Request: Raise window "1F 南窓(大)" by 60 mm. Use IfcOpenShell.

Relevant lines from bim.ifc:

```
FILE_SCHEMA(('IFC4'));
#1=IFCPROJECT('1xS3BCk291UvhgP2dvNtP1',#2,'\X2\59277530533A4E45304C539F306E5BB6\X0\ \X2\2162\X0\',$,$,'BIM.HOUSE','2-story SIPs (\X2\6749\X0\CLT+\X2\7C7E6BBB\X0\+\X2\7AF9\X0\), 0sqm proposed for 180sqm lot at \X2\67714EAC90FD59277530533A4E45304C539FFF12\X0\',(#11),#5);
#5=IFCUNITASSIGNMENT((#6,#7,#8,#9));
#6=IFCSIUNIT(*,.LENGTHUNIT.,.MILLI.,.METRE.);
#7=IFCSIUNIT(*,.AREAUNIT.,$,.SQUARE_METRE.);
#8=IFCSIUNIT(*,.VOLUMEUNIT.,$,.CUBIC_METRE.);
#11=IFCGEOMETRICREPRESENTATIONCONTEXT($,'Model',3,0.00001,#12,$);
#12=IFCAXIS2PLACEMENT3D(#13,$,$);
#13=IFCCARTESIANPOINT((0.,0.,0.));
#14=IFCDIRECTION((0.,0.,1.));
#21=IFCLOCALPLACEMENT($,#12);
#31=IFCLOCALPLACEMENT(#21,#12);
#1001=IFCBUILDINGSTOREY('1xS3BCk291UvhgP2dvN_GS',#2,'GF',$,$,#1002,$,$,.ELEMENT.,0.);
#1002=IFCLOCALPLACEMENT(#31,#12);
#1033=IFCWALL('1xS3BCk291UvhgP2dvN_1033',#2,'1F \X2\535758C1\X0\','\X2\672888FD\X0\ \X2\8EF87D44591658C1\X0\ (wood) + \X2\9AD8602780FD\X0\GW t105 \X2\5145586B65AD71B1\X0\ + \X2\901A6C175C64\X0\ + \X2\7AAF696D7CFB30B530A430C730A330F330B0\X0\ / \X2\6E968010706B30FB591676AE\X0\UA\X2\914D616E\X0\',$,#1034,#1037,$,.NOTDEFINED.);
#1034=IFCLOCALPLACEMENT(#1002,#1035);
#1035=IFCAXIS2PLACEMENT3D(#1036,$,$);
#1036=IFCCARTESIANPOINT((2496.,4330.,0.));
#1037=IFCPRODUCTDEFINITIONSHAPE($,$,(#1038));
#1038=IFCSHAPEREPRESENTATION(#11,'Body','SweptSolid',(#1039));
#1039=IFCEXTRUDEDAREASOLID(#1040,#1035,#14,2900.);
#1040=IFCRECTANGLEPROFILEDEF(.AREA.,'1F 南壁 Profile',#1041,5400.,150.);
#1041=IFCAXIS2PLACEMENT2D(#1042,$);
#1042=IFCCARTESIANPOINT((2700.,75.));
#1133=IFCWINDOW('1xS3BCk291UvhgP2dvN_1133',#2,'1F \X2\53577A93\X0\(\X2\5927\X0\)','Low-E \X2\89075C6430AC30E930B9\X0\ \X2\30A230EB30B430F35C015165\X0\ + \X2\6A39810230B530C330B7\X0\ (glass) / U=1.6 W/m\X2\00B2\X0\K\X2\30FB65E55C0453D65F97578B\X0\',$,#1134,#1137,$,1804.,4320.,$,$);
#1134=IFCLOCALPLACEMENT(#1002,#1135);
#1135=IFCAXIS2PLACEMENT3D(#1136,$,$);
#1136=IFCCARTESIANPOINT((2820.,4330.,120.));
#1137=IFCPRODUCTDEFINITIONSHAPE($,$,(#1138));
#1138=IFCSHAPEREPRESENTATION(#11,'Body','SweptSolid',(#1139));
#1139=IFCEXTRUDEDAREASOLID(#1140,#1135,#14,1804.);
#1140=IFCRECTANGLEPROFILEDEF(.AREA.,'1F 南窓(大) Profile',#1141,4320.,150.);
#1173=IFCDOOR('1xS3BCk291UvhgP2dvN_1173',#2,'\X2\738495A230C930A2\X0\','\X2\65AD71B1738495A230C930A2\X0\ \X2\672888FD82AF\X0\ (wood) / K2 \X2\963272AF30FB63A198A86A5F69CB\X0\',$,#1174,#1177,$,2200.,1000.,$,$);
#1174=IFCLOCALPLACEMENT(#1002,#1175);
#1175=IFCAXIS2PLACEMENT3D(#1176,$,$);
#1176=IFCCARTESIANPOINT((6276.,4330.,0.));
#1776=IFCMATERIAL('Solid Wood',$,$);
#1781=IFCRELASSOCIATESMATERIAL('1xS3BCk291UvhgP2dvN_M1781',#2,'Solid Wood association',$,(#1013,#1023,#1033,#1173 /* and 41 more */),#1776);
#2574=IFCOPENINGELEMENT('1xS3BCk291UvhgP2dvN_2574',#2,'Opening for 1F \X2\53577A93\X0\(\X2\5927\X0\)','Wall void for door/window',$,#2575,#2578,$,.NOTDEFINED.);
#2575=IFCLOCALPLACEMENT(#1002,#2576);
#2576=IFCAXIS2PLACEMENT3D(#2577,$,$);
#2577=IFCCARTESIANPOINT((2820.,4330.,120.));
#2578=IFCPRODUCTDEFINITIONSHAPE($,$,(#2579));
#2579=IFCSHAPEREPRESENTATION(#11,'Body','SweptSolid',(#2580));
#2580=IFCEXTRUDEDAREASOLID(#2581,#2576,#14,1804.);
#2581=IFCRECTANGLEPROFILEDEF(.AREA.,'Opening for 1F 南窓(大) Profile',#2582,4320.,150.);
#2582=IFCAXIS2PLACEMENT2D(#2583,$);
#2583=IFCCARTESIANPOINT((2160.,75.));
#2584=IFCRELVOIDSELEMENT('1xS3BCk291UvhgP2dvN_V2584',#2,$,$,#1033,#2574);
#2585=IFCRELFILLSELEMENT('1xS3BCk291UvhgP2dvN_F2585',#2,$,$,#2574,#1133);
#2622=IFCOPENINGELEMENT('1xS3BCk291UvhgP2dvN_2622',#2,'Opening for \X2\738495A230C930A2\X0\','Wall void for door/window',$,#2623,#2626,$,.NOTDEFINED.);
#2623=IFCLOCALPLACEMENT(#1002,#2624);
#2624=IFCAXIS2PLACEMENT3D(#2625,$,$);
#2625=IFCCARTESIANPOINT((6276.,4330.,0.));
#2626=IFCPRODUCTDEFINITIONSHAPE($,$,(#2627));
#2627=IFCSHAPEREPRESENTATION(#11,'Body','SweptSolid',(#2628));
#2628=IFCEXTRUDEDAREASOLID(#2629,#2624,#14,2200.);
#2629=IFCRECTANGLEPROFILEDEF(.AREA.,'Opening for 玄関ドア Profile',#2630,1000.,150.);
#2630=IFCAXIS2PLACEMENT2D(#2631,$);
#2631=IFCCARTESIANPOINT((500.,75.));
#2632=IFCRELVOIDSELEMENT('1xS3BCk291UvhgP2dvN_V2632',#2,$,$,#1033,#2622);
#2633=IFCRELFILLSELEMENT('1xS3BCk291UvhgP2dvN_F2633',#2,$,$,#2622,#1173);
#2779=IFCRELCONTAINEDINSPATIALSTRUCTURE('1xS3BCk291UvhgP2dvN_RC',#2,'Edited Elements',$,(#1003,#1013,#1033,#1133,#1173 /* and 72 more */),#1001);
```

```python
import numpy as np
import ifcopenshell
import ifcopenshell.api.geometry
import ifcopenshell.util.placement
import ifcopenshell.util.unit

model = ifcopenshell.open("bim.ifc")
unit_scale = ifcopenshell.util.unit.calculate_unit_scale(model)

window = model.by_id(1133)
opening = window.FillsVoids[0].RelatingOpeningElement
dz = 0.06 / unit_scale

shift = np.array([0.0, 0.0, dz])
# The window is not placed relative to its opening, so move both.
for product in (opening, window):
    matrix = ifcopenshell.util.placement.get_local_placement(product.ObjectPlacement)
    matrix[:3, 3] += shift
    ifcopenshell.api.geometry.edit_object_placement(model, product=product, matrix=matrix, is_si=False)

print(f"moved by {dz * unit_scale:+.3f} m")

model.write("bim_rev.ifc")
```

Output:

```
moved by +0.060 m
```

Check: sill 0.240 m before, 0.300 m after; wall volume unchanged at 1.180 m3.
